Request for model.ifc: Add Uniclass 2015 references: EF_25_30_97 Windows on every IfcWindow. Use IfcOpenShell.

First a look at what the model holds.

```python
import ifcopenshell

model = ifcopenshell.open("model.ifc")
print(model.schema)
print("classifications:", [c.Name for c in model.by_type("IfcClassification")])
for ifc_class in ("IfcDoor", "IfcRoof", "IfcStair", "IfcWall", "IfcWindow"):
    print(ifc_class, len(model.by_type(ifc_class)))
```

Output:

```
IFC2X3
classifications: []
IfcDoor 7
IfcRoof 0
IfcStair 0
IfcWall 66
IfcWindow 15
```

```python
import ifcopenshell
import ifcopenshell.api.classification

model = ifcopenshell.open("model.ifc")

# IFC2X3 requires Source and Edition and has no link from the project to the system.
system = model.create_entity("IfcClassification", Source="NBS", Edition="2015", Name="Uniclass 2015")

codes = {
    "IfcWindow": ("EF_25_30_97", "Windows"),
}
for ifc_class, (code, name) in codes.items():
    products = model.by_type(ifc_class)
    ifcopenshell.api.classification.add_reference(
        model, products=products, classification=system, identification=code, name=name
    )
    print(code, len(products))

model.write("model_rev.ifc")
```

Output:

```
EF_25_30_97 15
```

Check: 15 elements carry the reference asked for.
